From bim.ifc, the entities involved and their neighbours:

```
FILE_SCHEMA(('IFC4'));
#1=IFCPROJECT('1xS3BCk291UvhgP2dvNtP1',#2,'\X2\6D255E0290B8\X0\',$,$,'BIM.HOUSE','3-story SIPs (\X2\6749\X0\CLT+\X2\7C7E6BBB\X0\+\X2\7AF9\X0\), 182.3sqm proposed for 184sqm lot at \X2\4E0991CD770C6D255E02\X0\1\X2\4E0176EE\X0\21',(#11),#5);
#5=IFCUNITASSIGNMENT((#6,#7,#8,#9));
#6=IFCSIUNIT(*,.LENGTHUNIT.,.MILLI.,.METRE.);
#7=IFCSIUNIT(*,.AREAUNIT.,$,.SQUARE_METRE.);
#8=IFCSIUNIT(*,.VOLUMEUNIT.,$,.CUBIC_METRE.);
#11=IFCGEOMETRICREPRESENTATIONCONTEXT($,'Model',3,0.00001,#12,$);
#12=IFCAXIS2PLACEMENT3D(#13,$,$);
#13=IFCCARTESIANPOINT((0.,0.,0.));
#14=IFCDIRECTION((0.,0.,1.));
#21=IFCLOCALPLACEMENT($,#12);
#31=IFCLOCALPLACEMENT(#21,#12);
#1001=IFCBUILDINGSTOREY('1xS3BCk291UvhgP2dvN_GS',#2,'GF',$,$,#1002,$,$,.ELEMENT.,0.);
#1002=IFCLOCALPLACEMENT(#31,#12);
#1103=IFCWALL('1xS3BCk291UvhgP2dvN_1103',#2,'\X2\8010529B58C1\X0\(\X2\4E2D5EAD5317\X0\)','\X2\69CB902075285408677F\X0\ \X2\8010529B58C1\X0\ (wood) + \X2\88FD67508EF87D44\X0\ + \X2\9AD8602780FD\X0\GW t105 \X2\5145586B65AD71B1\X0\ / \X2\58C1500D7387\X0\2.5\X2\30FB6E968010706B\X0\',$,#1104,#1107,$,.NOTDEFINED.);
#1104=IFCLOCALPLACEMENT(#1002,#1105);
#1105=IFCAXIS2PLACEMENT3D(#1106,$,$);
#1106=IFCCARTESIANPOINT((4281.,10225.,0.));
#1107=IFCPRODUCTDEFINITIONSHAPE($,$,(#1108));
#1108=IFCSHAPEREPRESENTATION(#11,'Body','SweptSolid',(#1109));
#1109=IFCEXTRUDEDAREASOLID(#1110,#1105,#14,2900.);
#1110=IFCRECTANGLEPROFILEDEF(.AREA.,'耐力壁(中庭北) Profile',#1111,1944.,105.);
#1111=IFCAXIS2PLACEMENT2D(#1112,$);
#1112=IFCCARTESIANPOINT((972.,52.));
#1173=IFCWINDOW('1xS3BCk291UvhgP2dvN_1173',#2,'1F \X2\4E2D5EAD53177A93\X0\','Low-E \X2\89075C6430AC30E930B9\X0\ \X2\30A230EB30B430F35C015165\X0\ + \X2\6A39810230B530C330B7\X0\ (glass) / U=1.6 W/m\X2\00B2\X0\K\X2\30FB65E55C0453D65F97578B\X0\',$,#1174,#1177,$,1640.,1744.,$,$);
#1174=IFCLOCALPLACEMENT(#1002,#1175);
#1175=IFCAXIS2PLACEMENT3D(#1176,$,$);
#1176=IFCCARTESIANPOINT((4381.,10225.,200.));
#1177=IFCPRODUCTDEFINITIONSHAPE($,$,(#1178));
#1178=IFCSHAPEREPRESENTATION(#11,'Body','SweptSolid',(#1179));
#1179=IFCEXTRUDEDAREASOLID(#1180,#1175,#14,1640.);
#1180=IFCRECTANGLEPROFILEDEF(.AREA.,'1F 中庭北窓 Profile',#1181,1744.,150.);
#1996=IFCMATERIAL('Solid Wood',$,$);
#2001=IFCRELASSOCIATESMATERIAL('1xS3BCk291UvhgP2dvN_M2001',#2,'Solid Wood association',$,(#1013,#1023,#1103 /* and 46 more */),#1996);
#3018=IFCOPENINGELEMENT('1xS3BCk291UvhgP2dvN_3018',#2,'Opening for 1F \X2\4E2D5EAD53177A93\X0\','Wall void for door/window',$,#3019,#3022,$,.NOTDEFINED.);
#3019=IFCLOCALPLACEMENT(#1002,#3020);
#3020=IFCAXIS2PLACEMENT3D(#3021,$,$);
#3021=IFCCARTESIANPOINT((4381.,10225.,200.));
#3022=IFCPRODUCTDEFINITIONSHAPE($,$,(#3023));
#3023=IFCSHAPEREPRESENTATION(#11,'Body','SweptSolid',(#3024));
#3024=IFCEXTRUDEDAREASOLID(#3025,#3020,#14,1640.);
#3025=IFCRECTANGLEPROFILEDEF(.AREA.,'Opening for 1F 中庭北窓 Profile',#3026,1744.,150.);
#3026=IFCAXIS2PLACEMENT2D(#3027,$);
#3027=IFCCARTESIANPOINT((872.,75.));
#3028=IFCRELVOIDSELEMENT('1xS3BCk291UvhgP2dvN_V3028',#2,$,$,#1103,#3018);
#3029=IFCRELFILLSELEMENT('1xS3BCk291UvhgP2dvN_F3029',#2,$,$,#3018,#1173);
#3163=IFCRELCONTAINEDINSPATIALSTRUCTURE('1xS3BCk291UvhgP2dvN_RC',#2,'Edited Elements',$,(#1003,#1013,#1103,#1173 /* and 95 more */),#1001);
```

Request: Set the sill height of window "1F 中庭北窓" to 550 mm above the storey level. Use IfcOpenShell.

```python
import numpy as np
import ifcopenshell
import ifcopenshell.api.geometry
import ifcopenshell.geom
import ifcopenshell.util.element
import ifcopenshell.util.placement
import ifcopenshell.util.shape
import ifcopenshell.util.unit

model = ifcopenshell.open("bim.ifc")
unit_scale = ifcopenshell.util.unit.calculate_unit_scale(model)

window = model.by_guid("1xS3BCk291UvhgP2dvN_1173")
opening = window.FillsVoids[0].RelatingOpeningElement
storey = ifcopenshell.util.element.get_container(window, ifc_class="IfcBuildingStorey")
level = ifcopenshell.util.placement.get_local_placement(storey.ObjectPlacement)[2, 3]

# The opening's origin need not be at the sill, so measure its lowest point.
shape = ifcopenshell.geom.create_shape(ifcopenshell.geom.settings(), opening)
bottom = ifcopenshell.util.shape.get_shape_bottom_elevation(shape, shape.geometry) / unit_scale
dz = level + 0.55 / unit_scale - bottom

shift = np.array([0.0, 0.0, dz])
# The window is not placed relative to its opening, so move both.
for product in (opening, window):
    matrix = ifcopenshell.util.placement.get_local_placement(product.ObjectPlacement)
    matrix[:3, 3] += shift
    ifcopenshell.api.geometry.edit_object_placement(model, product=product, matrix=matrix, is_si=False)

print(f"moved by {dz * unit_scale:+.3f} m")

model.write("bim_rev.ifc")
```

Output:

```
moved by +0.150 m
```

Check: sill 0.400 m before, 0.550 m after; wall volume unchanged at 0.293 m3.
